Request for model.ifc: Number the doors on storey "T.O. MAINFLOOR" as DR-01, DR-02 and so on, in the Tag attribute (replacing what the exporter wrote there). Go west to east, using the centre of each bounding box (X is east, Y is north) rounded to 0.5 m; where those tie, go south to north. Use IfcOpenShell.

First a look at what the model holds.

```python
import ifcopenshell
import ifcopenshell.util.element
import ifcopenshell.util.placement

model = ifcopenshell.open("model.ifc")
print(model.schema)
storey = next(s for s in model.by_type("IfcBuildingStorey") if s.Name == "T.O. MAINFLOOR")
doors = [e for e in ifcopenshell.util.element.get_decomposition(storey) if e.is_a("IfcDoor")]
for e in sorted(doors, key=lambda e: e.id()):
    origin = ifcopenshell.util.placement.get_local_placement(e.ObjectPlacement)[:3, 3]
    print(e.id(), e.Tag, e.Name, origin.round(2) + 0.0, sep=" | ")
```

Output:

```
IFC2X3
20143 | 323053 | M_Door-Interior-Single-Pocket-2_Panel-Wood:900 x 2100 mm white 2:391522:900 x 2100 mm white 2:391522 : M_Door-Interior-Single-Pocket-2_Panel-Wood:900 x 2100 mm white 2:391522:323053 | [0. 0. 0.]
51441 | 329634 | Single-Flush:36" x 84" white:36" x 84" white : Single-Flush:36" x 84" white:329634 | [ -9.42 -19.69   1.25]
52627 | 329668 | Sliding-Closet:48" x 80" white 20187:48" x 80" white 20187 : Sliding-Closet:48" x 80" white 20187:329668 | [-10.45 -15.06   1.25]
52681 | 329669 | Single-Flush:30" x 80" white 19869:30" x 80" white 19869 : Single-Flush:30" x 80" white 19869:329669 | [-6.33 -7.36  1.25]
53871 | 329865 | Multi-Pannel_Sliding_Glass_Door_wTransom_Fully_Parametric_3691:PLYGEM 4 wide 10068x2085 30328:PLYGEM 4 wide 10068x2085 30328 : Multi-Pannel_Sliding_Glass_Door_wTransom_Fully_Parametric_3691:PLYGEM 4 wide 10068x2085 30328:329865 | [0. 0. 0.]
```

```python
import ifcopenshell
import ifcopenshell.geom
import ifcopenshell.util.element
import ifcopenshell.util.shape

model = ifcopenshell.open("model.ifc")
settings = ifcopenshell.geom.settings()
settings.set("use-world-coords", True)


def centre(element):
    shape = ifcopenshell.geom.create_shape(settings, element)
    return ifcopenshell.util.shape.get_bbox_centroid(shape.geometry)


storey = next(s for s in model.by_type("IfcBuildingStorey") if s.Name == "T.O. MAINFLOOR")
doors = [e for e in ifcopenshell.util.element.get_decomposition(storey) if e.is_a("IfcDoor")]

# Insertion points can sit at a corner or the storey origin, so sort by the geometry (in metres).
centres = {e: centre(e) for e in doors}
doors.sort(key=lambda e: (round(centres[e][0] / 0.5), centres[e][1]))

for i, e in enumerate(doors, start=1):
    number = f"DR-{i:02d}"
    e.Tag = number
    print(e.id(), number)

model.write("model_edited.ifc")
```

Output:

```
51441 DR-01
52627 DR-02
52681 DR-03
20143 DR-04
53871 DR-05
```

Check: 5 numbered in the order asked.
